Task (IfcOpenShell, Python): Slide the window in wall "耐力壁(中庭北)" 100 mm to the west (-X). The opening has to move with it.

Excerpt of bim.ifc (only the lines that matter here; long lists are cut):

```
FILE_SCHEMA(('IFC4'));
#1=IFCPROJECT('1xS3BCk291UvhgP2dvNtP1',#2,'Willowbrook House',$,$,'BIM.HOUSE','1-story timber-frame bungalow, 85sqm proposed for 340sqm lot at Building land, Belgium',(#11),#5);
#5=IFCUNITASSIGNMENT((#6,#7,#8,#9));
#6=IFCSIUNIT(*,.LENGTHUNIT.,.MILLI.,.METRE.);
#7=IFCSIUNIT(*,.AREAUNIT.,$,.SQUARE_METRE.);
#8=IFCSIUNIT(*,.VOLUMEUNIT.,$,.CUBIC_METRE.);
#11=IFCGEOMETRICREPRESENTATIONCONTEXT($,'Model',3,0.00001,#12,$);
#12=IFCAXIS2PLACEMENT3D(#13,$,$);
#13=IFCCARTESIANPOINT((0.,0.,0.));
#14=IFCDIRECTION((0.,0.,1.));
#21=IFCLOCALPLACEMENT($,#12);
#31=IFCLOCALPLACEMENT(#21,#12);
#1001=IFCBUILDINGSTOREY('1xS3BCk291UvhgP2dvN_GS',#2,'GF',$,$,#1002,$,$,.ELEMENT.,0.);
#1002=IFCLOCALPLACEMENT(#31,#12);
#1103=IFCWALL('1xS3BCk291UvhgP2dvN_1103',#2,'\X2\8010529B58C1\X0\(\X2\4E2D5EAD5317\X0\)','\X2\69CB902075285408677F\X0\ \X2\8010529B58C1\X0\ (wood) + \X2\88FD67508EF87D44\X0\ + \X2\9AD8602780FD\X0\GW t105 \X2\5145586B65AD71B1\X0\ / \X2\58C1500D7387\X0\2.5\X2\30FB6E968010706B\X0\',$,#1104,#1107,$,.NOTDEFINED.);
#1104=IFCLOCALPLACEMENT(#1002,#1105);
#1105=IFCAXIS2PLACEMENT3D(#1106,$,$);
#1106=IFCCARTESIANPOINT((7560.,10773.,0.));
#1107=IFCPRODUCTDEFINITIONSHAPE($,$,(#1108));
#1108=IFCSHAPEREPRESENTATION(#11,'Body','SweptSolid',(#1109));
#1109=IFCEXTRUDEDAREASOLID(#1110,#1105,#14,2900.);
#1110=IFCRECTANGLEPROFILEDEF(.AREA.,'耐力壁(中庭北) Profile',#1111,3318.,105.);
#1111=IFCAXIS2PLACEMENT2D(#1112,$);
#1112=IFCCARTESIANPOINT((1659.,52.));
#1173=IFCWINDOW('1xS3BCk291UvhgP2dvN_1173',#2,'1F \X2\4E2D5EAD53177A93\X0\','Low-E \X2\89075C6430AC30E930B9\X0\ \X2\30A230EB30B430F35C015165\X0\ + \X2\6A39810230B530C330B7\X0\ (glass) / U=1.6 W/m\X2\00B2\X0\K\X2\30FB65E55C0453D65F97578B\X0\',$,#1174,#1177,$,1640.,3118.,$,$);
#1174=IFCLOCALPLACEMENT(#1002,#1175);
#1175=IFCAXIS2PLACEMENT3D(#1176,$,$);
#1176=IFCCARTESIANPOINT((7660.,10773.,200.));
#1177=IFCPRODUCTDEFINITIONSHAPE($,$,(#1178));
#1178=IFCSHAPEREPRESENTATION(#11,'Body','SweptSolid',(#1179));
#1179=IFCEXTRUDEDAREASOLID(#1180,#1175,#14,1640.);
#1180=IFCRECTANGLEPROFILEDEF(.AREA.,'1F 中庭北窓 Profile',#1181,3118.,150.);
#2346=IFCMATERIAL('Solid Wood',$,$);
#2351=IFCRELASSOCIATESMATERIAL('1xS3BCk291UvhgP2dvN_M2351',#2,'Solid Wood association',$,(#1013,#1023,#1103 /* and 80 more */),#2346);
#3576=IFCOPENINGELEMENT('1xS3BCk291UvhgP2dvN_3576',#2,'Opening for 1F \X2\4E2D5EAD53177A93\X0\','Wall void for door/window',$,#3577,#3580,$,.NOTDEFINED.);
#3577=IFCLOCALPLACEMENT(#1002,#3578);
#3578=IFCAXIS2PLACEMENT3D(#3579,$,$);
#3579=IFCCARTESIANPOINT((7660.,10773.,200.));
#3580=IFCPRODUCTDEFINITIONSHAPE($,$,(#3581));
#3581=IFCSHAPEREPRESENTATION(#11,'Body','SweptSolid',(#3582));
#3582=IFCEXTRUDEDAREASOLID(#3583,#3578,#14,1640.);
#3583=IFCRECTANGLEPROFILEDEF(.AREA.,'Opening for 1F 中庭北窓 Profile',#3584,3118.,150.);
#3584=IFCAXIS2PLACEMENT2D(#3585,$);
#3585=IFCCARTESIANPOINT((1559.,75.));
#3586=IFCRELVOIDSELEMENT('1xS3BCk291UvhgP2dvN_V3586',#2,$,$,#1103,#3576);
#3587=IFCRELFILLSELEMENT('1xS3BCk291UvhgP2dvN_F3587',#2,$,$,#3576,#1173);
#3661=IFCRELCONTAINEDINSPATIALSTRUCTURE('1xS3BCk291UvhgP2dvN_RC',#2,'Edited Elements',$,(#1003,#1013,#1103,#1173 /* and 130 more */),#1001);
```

```python
import ifcopenshell
import ifcopenshell.api.geometry
import ifcopenshell.util.placement
import ifcopenshell.util.unit

model = ifcopenshell.open("bim.ifc")
unit_scale = ifcopenshell.util.unit.calculate_unit_scale(model)

window = model.by_id(1173)
opening = window.FillsVoids[0].RelatingOpeningElement
wall = opening.VoidsElements[0].RelatingBuildingElement

wall_matrix = ifcopenshell.util.placement.get_local_placement(wall.ObjectPlacement)
shift = wall_matrix[:3, 0] * -0.1 / unit_scale
before = ifcopenshell.util.placement.get_local_placement(window.ObjectPlacement)[:3, 3].copy()

# The window is not placed relative to its opening, so move both.
for product in (opening, window):
    matrix = ifcopenshell.util.placement.get_local_placement(product.ObjectPlacement)
    matrix[:3, 3] += shift
    ifcopenshell.api.geometry.edit_object_placement(model, product=product, matrix=matrix, is_si=False)

after = ifcopenshell.util.placement.get_local_placement(window.ObjectPlacement)[:3, 3]
print("window moved by", (after - before).round(3) + 0.0)

model.write("bim_updated.ifc")
```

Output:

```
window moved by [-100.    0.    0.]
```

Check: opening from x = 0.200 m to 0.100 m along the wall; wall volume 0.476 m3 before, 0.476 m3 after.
